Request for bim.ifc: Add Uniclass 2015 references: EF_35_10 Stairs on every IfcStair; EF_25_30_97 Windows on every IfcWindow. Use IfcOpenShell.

First a look at what the model holds.

```python
import ifcopenshell

model = ifcopenshell.open("bim.ifc")
print(model.schema)
print("classifications:", [c.Name for c in model.by_type("IfcClassification")])
for ifc_class in ("IfcDoor", "IfcRoof", "IfcStair", "IfcWall", "IfcWindow"):
    print(ifc_class, len(model.by_type(ifc_class)))
```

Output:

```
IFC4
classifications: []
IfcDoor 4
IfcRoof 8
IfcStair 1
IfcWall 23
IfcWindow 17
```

```python
import ifcopenshell
import ifcopenshell.api.classification

model = ifcopenshell.open("bim.ifc")

system = ifcopenshell.api.classification.add_classification(model, classification="Uniclass 2015")

codes = {
    "IfcStair": ("EF_35_10", "Stairs"),
    "IfcWindow": ("EF_25_30_97", "Windows"),
}
for ifc_class, (code, name) in codes.items():
    products = model.by_type(ifc_class)
    ifcopenshell.api.classification.add_reference(
        model, products=products, classification=system, identification=code, name=name
    )
    print(code, len(products))

model.write("bim_rev.ifc")
```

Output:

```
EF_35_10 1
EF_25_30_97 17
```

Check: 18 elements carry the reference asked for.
